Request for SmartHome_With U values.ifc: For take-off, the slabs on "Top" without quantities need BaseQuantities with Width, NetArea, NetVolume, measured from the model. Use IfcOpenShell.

First a look at what the model holds.

```python
import ifcopenshell
import ifcopenshell.util.element
import ifcopenshell.util.unit

model = ifcopenshell.open("SmartHome_With U values.ifc")
print(model.schema)
for unit_type in ("LENGTHUNIT", "AREAUNIT", "VOLUMEUNIT"):
    print(unit_type, ifcopenshell.util.unit.calculate_unit_scale(model, unit_type))
storey = next(s for s in model.by_type("IfcBuildingStorey") if s.Name == "Top")
slabs = [e for e in ifcopenshell.util.element.get_decomposition(storey) if e.is_a("IfcSlab")]
for e in sorted(slabs, key=lambda e: e.id()):
    print(e.id(), e.is_a(), e.Name, list(ifcopenshell.util.element.get_psets(e, qtos_only=True)), sep=" | ")
```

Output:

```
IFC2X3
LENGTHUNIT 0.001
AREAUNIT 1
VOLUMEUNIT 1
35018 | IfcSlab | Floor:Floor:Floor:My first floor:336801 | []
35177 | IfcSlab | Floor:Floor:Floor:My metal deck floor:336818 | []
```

```python
import ifcopenshell
import ifcopenshell.api.pset
import ifcopenshell.geom
import ifcopenshell.util.element
import ifcopenshell.util.shape
import ifcopenshell.util.unit

model = ifcopenshell.open("SmartHome_With U values.ifc")
unit_scale = ifcopenshell.util.unit.calculate_unit_scale(model)
area_scale = ifcopenshell.util.unit.calculate_unit_scale(model, "AREAUNIT")
volume_scale = ifcopenshell.util.unit.calculate_unit_scale(model, "VOLUMEUNIT")
settings = ifcopenshell.geom.settings()

storey = next(s for s in model.by_type("IfcBuildingStorey") if s.Name == "Top")
slabs = [e for e in ifcopenshell.util.element.get_decomposition(storey) if e.is_a("IfcSlab")]

for e in sorted(slabs, key=lambda e: e.id()):
    if ifcopenshell.util.element.get_psets(e, qtos_only=True, should_inherit=False):
        continue
    # Geometry comes back in metres, in the element's own axes.
    shape = ifcopenshell.geom.create_shape(settings, e)
    values = {
        "Width": ifcopenshell.util.shape.get_z(shape.geometry) / unit_scale,
        "NetArea": ifcopenshell.util.shape.get_footprint_area(shape.geometry) / area_scale,
        "NetVolume": ifcopenshell.util.shape.get_volume(shape.geometry) / volume_scale,
    }
    qto = ifcopenshell.api.pset.add_qto(model, product=e, name="BaseQuantities")
    ifcopenshell.api.pset.edit_qto(model, qto=qto, properties=values)
    print(e.id(), {k: round(v, 3) for k, v in values.items()})

model.write("SmartHome_With U values_updated.ifc")
```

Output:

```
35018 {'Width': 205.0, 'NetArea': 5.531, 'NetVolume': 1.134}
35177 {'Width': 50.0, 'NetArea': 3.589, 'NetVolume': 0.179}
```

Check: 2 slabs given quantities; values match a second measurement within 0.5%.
